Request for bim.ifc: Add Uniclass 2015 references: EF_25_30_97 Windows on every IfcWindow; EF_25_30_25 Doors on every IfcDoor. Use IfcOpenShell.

First a look at what the model holds.

```python
import ifcopenshell

model = ifcopenshell.open("bim.ifc")
print(model.schema)
print("classifications:", [c.Name for c in model.by_type("IfcClassification")])
for ifc_class in ("IfcDoor", "IfcRoof", "IfcStair", "IfcWall", "IfcWindow"):
    print(ifc_class, len(model.by_type(ifc_class)))
```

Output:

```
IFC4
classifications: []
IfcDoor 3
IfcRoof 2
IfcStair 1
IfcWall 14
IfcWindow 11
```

```python
import ifcopenshell
import ifcopenshell.api.classification

model = ifcopenshell.open("bim.ifc")

system = ifcopenshell.api.classification.add_classification(model, classification="Uniclass 2015")

codes = {
    "IfcWindow": ("EF_25_30_97", "Windows"),
    "IfcDoor": ("EF_25_30_25", "Doors"),
}
for ifc_class, (code, name) in codes.items():
    products = model.by_type(ifc_class)
    ifcopenshell.api.classification.add_reference(
        model, products=products, classification=system, identification=code, name=name
    )
    print(code, len(products))

model.write("bim_v2.ifc")
```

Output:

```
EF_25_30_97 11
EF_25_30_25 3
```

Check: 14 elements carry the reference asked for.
